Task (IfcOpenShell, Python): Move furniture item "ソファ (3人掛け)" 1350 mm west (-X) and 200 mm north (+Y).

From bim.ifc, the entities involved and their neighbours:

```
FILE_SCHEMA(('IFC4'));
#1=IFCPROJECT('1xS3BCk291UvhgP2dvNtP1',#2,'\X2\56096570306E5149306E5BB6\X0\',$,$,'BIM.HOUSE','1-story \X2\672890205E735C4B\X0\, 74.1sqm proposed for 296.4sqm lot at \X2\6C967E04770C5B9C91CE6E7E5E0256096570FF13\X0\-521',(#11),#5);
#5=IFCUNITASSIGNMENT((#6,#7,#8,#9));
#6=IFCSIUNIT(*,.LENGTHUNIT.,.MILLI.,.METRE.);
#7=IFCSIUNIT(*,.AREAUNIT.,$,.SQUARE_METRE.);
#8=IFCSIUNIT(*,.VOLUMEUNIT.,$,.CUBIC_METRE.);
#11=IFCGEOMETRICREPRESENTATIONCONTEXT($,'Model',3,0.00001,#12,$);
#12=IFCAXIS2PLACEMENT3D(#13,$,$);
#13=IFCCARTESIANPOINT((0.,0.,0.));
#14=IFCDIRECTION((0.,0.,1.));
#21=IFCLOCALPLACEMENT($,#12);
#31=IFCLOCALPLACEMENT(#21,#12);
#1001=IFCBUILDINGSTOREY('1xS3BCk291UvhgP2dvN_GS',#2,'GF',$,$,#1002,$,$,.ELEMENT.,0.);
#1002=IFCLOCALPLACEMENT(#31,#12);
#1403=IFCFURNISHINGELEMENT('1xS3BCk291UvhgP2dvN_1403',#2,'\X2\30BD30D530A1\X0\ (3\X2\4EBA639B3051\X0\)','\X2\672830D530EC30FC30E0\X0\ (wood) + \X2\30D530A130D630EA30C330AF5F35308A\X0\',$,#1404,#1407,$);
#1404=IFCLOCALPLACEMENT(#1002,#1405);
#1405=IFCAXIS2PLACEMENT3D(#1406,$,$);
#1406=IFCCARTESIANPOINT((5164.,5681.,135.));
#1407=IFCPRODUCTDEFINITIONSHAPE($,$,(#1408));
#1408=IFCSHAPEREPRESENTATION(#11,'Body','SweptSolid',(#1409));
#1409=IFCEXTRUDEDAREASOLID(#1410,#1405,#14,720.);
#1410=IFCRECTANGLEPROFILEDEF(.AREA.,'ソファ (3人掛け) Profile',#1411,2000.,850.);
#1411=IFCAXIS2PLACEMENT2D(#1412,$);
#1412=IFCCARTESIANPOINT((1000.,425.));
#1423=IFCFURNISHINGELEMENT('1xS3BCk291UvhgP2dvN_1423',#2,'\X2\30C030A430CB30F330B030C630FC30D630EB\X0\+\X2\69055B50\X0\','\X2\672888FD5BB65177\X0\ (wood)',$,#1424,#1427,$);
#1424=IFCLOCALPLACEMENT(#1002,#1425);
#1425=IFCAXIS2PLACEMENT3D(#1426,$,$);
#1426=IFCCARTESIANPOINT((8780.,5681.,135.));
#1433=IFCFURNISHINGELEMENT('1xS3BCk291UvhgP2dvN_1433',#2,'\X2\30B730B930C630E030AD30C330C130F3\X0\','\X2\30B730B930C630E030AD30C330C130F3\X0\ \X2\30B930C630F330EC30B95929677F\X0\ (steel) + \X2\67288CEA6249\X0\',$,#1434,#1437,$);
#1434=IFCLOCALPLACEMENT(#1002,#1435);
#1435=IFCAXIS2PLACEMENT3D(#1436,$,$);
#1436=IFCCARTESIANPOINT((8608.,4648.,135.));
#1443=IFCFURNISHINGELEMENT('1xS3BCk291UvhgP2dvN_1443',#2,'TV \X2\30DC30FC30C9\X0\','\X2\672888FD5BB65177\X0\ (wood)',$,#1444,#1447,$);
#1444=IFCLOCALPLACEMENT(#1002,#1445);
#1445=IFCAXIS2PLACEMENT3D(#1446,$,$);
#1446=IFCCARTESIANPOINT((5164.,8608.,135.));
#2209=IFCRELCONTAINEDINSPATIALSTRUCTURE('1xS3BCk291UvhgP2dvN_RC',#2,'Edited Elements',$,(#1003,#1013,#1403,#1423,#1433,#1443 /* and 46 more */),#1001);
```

```python
import ifcopenshell
import ifcopenshell.api.geometry
import ifcopenshell.util.placement

model = ifcopenshell.open("bim.ifc")

item = model.by_guid("1xS3BCk291UvhgP2dvN_1403")
matrix = ifcopenshell.util.placement.get_local_placement(item.ObjectPlacement)
matrix[0, 3] -= 1350.0
matrix[1, 3] += 200.0
ifcopenshell.api.geometry.edit_object_placement(model, product=item, matrix=matrix, is_si=False)

print(ifcopenshell.util.placement.get_local_placement(item.ObjectPlacement).round(3) + 0.0)

model.write("bim_rev.ifc")
```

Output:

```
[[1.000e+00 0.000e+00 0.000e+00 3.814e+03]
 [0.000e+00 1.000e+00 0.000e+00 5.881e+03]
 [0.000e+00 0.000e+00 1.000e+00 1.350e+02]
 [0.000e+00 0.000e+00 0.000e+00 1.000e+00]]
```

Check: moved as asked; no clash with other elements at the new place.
